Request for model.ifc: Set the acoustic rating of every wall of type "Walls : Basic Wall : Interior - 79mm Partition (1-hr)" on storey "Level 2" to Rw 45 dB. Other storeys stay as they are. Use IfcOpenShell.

First a look at what the model holds.

```python
import ifcopenshell
import ifcopenshell.util.element

model = ifcopenshell.open("model.ifc")
print(model.schema)
storey = next(s for s in model.by_type("IfcBuildingStorey") if s.Name == "Level 2")
walls = [e for e in ifcopenshell.util.element.get_decomposition(storey) if e.is_a("IfcWall")]
seen = {}
for e in walls:
    element_type = ifcopenshell.util.element.get_type(e)
    key = (element_type.Name if element_type != e and element_type else None, ifcopenshell.util.element.get_pset(e, "Pset_WallCommon", "AcousticRating"))
    seen[key] = seen.get(key, 0) + 1
for (name, value), count in sorted(seen.items(), key=str):
    print(count, "x", name, "|", value)
```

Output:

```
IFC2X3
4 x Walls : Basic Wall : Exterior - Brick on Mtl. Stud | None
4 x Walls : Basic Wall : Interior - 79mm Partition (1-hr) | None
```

```python
import ifcopenshell
import ifcopenshell.api.pset
import ifcopenshell.util.element

model = ifcopenshell.open("model.ifc")

storey = next(s for s in model.by_type("IfcBuildingStorey") if s.Name == "Level 2")
walls = [e for e in ifcopenshell.util.element.get_decomposition(storey) if e.is_a("IfcWall")]

count = 0
for e in walls:
    element_type = ifcopenshell.util.element.get_type(e)
    if element_type in (None, e) or element_type.Name != "Walls : Basic Wall : Interior - 79mm Partition (1-hr)":
        continue
    # add_pset returns the element's existing set when there is one.
    pset = ifcopenshell.api.pset.add_pset(model, product=e, name="Pset_WallCommon")
    ifcopenshell.api.pset.edit_pset(model, pset=pset, properties={"AcousticRating": "Rw 45 dB"})
    count += 1

print(count, "walls updated")

model.write("model_updated.ifc")
```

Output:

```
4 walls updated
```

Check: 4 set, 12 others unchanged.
